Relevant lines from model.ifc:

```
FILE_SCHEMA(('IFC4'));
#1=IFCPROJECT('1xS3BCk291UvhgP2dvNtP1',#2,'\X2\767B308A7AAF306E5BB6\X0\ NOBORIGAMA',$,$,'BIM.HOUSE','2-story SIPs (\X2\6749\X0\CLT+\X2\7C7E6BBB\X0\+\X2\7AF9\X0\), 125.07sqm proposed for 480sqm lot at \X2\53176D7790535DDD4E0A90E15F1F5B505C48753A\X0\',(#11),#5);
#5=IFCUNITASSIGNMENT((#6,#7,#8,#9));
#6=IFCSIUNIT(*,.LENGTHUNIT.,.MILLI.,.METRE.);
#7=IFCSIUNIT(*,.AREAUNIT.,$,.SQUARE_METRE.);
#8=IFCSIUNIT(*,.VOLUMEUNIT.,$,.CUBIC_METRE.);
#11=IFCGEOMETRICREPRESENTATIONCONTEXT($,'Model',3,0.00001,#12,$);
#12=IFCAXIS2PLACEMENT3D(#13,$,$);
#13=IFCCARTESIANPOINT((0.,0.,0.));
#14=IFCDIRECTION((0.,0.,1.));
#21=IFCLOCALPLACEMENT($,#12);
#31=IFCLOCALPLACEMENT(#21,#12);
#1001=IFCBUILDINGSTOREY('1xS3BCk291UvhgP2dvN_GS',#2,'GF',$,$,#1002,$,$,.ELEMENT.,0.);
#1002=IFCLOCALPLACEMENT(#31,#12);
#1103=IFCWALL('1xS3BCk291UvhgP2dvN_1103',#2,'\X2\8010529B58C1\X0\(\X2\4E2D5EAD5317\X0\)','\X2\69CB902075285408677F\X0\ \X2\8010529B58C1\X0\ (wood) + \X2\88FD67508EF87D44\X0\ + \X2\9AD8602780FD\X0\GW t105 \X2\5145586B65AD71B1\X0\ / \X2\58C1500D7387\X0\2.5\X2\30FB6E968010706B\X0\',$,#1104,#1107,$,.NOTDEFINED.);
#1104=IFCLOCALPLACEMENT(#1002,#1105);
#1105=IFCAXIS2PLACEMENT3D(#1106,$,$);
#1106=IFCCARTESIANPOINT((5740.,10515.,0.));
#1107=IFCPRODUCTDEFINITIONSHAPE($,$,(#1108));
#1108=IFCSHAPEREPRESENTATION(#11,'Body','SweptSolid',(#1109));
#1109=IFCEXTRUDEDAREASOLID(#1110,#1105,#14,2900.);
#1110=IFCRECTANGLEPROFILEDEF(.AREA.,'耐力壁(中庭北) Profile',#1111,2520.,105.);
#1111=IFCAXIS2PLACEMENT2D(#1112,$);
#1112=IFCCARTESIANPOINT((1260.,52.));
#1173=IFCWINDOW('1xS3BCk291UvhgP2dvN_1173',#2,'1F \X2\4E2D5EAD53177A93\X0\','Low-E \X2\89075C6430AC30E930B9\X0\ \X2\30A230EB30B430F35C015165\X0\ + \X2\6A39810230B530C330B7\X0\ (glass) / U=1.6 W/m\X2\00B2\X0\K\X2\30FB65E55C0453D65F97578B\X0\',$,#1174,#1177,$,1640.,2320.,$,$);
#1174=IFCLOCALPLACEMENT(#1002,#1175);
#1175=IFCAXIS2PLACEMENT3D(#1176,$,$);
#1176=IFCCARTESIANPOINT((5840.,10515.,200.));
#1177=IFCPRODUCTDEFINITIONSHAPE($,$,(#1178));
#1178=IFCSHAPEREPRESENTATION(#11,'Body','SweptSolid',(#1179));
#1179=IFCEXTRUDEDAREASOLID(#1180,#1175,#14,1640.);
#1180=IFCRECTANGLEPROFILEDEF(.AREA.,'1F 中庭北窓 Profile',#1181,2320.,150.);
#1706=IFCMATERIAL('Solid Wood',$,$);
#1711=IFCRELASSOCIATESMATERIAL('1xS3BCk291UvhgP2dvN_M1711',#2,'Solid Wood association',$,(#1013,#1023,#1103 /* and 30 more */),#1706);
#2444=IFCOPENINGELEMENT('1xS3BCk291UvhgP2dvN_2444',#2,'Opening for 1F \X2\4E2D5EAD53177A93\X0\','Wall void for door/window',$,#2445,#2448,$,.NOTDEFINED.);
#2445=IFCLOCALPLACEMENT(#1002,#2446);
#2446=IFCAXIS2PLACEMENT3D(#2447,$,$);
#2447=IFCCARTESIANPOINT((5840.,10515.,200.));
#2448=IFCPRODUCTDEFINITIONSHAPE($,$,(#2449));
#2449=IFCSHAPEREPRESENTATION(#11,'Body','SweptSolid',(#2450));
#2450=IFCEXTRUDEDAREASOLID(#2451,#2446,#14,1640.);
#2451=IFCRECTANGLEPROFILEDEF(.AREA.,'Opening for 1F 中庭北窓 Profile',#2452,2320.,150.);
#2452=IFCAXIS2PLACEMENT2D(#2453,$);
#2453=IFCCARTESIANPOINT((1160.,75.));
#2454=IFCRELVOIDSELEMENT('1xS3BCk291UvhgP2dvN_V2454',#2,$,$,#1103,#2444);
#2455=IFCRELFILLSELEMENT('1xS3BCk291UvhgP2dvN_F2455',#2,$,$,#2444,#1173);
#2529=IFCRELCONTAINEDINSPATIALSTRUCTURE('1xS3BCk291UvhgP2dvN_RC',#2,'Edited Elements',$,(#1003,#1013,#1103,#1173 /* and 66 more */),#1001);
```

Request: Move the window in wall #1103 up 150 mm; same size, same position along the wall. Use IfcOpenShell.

```python
import numpy as np
import ifcopenshell
import ifcopenshell.api.geometry
import ifcopenshell.util.placement
import ifcopenshell.util.unit

model = ifcopenshell.open("model.ifc")
unit_scale = ifcopenshell.util.unit.calculate_unit_scale(model)

window = model.by_guid("1xS3BCk291UvhgP2dvN_1173")
opening = window.FillsVoids[0].RelatingOpeningElement
dz = 0.15 / unit_scale

shift = np.array([0.0, 0.0, dz])
# The window is not placed relative to its opening, so move both.
for product in (opening, window):
    matrix = ifcopenshell.util.placement.get_local_placement(product.ObjectPlacement)
    matrix[:3, 3] += shift
    ifcopenshell.api.geometry.edit_object_placement(model, product=product, matrix=matrix, is_si=False)

print(f"moved by {dz * unit_scale:+.3f} m")

model.write("model_edited.ifc")
```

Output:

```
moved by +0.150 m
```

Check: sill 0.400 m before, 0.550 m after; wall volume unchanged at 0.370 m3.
